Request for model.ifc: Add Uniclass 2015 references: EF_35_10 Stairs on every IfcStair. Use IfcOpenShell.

First a look at what the model holds.

```python
import ifcopenshell

model = ifcopenshell.open("model.ifc")
print(model.schema)
print("classifications:", [c.Name for c in model.by_type("IfcClassification")])
for ifc_class in ("IfcDoor", "IfcRoof", "IfcStair", "IfcWall", "IfcWindow"):
    print(ifc_class, len(model.by_type(ifc_class)))
```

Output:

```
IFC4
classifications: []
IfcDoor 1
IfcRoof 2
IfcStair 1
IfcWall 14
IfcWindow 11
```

```python
import ifcopenshell
import ifcopenshell.api.classification

model = ifcopenshell.open("model.ifc")

system = ifcopenshell.api.classification.add_classification(model, classification="Uniclass 2015")

codes = {
    "IfcStair": ("EF_35_10", "Stairs"),
}
for ifc_class, (code, name) in codes.items():
    products = model.by_type(ifc_class)
    ifcopenshell.api.classification.add_reference(
        model, products=products, classification=system, identification=code, name=name
    )
    print(code, len(products))

model.write("model_updated.ifc")
```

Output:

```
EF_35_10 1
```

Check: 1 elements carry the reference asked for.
